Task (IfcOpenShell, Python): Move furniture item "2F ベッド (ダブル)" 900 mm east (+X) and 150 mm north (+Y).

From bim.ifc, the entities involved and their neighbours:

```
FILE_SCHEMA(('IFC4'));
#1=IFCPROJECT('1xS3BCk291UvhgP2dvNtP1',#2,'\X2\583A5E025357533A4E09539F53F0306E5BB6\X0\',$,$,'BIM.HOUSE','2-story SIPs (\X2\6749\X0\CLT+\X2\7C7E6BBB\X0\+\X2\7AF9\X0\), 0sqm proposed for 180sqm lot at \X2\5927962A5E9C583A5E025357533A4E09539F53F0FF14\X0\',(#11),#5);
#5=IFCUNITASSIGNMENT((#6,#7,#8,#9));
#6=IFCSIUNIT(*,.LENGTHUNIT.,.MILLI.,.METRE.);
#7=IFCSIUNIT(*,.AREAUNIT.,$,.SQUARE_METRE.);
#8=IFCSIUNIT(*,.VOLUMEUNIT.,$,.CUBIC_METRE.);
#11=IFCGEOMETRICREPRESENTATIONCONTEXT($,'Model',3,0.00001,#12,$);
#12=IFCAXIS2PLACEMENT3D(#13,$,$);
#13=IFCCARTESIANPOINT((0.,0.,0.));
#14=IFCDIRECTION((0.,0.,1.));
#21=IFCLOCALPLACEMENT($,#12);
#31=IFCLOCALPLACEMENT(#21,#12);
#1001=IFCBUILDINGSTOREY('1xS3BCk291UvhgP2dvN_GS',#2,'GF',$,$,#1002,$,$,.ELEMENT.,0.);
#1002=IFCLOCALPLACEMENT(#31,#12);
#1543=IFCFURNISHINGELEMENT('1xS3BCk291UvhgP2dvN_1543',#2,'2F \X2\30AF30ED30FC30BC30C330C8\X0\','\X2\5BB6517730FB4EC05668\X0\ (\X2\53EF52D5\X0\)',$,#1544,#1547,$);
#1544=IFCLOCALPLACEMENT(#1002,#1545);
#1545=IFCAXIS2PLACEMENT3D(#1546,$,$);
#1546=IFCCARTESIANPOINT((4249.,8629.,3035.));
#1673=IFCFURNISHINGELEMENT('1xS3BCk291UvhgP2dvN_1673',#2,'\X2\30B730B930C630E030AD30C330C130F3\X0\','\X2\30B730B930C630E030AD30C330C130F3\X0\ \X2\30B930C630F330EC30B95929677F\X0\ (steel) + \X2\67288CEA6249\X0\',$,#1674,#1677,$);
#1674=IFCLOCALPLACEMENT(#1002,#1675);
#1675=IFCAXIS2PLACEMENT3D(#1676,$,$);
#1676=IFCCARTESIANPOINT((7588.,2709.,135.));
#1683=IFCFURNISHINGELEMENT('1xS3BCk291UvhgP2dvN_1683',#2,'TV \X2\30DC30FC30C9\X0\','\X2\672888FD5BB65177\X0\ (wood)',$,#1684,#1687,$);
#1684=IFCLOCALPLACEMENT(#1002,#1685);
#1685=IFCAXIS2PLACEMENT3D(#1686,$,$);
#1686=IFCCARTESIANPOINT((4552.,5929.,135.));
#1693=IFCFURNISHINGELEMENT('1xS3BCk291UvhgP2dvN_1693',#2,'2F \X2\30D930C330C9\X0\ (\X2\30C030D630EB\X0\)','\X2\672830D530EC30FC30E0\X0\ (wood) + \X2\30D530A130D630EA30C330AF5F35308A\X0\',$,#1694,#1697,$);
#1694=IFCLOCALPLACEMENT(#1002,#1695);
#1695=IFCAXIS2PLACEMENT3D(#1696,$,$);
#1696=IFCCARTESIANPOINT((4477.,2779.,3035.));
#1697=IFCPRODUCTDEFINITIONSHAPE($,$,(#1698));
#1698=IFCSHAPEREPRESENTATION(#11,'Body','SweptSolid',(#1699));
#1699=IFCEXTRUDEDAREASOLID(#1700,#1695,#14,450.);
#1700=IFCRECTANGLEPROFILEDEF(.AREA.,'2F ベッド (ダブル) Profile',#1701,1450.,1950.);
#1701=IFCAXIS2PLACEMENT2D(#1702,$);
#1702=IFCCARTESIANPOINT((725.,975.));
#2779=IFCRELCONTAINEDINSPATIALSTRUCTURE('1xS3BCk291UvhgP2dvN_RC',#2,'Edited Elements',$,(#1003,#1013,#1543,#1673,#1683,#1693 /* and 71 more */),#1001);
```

```python
import ifcopenshell
import ifcopenshell.api.geometry
import ifcopenshell.util.placement

model = ifcopenshell.open("bim.ifc")

item = model.by_id(1693)
matrix = ifcopenshell.util.placement.get_local_placement(item.ObjectPlacement)
matrix[0, 3] += 900.0
matrix[1, 3] += 150.0
ifcopenshell.api.geometry.edit_object_placement(model, product=item, matrix=matrix, is_si=False)

print(ifcopenshell.util.placement.get_local_placement(item.ObjectPlacement).round(3) + 0.0)

model.write("bim_updated.ifc")
```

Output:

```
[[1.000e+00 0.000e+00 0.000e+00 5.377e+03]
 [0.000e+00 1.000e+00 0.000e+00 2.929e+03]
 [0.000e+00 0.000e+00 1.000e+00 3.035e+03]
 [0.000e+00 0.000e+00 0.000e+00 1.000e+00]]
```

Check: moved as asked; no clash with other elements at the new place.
